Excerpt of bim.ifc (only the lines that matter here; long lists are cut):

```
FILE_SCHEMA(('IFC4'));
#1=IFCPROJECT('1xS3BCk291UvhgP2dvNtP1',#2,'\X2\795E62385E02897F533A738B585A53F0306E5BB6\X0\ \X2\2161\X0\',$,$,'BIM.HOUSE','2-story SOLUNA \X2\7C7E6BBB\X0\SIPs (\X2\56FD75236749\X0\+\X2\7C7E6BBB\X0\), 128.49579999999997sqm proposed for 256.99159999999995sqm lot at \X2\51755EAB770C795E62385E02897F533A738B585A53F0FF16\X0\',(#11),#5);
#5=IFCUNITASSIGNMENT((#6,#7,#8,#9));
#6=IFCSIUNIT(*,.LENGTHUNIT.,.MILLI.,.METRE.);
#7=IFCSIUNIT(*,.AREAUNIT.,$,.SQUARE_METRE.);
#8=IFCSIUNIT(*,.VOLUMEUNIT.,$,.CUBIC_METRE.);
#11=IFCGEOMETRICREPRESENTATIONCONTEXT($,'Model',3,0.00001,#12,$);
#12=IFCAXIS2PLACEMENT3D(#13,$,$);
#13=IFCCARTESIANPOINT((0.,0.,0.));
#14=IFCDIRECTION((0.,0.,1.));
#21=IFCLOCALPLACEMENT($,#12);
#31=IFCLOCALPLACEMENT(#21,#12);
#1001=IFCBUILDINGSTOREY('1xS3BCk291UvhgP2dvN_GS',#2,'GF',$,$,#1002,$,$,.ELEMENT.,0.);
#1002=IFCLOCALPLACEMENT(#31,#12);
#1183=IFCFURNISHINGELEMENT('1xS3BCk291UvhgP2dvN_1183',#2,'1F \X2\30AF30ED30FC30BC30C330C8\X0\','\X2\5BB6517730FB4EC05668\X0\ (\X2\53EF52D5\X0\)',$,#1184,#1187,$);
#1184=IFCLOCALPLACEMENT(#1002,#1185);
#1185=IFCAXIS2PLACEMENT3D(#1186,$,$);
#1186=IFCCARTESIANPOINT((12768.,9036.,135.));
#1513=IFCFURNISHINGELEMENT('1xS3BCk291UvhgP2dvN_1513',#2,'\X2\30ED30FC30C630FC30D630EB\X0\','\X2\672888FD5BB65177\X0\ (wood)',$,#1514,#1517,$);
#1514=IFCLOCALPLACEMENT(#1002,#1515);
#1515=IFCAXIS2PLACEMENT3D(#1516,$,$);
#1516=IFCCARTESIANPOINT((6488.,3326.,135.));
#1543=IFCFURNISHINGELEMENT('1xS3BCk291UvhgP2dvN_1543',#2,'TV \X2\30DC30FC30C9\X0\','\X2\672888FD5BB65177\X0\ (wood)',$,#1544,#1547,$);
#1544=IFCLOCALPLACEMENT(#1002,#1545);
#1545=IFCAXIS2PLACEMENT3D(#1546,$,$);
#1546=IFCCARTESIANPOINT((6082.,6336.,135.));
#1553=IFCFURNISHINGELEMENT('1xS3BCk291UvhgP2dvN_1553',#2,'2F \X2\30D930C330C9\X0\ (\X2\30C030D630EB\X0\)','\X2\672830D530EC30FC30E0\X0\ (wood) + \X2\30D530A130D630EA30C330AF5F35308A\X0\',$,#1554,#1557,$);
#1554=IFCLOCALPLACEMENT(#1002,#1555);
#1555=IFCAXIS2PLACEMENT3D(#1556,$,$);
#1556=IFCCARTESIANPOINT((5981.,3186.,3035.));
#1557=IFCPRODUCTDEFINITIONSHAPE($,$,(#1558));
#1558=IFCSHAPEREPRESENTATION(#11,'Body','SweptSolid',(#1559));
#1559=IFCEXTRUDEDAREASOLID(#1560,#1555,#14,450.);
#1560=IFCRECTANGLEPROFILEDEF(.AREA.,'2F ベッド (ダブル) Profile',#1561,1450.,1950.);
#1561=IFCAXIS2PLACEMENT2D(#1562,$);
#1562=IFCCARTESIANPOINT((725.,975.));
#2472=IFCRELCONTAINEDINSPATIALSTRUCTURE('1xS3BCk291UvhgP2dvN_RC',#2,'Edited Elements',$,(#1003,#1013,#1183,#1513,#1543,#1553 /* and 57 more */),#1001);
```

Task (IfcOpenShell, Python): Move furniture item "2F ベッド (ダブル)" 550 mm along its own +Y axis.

```python
import ifcopenshell
import ifcopenshell.api.geometry
import ifcopenshell.util.placement
import ifcopenshell.util.unit

model = ifcopenshell.open("bim.ifc")
unit_scale = ifcopenshell.util.unit.calculate_unit_scale(model)

item = model.by_guid("1xS3BCk291UvhgP2dvN_1553")
matrix = ifcopenshell.util.placement.get_local_placement(item.ObjectPlacement)
matrix[:3, 3] += matrix[:3, 1] * 0.55 / unit_scale
ifcopenshell.api.geometry.edit_object_placement(model, product=item, matrix=matrix, is_si=False)

print(ifcopenshell.util.placement.get_local_placement(item.ObjectPlacement).round(3) + 0.0)

model.write("bim_edited.ifc")
```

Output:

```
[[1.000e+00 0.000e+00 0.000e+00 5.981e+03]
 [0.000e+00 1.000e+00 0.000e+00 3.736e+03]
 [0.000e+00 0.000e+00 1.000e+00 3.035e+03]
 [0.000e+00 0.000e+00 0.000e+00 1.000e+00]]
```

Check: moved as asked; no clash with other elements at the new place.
